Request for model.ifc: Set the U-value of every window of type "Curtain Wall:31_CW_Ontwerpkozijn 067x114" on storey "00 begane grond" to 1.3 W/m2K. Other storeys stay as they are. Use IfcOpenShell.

First a look at what the model holds.

```python
import ifcopenshell
import ifcopenshell.util.element

model = ifcopenshell.open("model.ifc")
print(model.schema)
storey = next(s for s in model.by_type("IfcBuildingStorey") if s.Name == "00 begane grond")
windows = [e for e in ifcopenshell.util.element.get_decomposition(storey) if e.is_a("IfcWindow")]
seen = {}
for e in windows:
    element_type = ifcopenshell.util.element.get_type(e)
    key = (element_type.Name if element_type != e and element_type else None, ifcopenshell.util.element.get_pset(e, "Pset_WindowCommon", "ThermalTransmittance"))
    seen[key] = seen.get(key, 0) + 1
for (name, value), count in sorted(seen.items(), key=str):
    print(count, "x", name, "|", value)
```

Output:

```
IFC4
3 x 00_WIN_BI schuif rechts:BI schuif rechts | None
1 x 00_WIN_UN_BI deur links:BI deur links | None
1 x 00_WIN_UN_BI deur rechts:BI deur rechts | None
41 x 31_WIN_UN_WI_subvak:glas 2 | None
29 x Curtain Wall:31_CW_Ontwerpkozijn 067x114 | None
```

```python
import ifcopenshell
import ifcopenshell.api.pset
import ifcopenshell.util.element

model = ifcopenshell.open("model.ifc")

storey = next(s for s in model.by_type("IfcBuildingStorey") if s.Name == "00 begane grond")
windows = [e for e in ifcopenshell.util.element.get_decomposition(storey) if e.is_a("IfcWindow")]

count = 0
for e in windows:
    element_type = ifcopenshell.util.element.get_type(e)
    if element_type in (None, e) or element_type.Name != "Curtain Wall:31_CW_Ontwerpkozijn 067x114":
        continue
    # add_pset returns the element's existing set when there is one.
    pset = ifcopenshell.api.pset.add_pset(model, product=e, name="Pset_WindowCommon")
    ifcopenshell.api.pset.edit_pset(model, pset=pset, properties={"ThermalTransmittance": 1.3})
    count += 1

print(count, "windows updated")

model.write("model_edited.ifc")
```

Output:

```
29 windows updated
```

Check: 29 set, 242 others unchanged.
